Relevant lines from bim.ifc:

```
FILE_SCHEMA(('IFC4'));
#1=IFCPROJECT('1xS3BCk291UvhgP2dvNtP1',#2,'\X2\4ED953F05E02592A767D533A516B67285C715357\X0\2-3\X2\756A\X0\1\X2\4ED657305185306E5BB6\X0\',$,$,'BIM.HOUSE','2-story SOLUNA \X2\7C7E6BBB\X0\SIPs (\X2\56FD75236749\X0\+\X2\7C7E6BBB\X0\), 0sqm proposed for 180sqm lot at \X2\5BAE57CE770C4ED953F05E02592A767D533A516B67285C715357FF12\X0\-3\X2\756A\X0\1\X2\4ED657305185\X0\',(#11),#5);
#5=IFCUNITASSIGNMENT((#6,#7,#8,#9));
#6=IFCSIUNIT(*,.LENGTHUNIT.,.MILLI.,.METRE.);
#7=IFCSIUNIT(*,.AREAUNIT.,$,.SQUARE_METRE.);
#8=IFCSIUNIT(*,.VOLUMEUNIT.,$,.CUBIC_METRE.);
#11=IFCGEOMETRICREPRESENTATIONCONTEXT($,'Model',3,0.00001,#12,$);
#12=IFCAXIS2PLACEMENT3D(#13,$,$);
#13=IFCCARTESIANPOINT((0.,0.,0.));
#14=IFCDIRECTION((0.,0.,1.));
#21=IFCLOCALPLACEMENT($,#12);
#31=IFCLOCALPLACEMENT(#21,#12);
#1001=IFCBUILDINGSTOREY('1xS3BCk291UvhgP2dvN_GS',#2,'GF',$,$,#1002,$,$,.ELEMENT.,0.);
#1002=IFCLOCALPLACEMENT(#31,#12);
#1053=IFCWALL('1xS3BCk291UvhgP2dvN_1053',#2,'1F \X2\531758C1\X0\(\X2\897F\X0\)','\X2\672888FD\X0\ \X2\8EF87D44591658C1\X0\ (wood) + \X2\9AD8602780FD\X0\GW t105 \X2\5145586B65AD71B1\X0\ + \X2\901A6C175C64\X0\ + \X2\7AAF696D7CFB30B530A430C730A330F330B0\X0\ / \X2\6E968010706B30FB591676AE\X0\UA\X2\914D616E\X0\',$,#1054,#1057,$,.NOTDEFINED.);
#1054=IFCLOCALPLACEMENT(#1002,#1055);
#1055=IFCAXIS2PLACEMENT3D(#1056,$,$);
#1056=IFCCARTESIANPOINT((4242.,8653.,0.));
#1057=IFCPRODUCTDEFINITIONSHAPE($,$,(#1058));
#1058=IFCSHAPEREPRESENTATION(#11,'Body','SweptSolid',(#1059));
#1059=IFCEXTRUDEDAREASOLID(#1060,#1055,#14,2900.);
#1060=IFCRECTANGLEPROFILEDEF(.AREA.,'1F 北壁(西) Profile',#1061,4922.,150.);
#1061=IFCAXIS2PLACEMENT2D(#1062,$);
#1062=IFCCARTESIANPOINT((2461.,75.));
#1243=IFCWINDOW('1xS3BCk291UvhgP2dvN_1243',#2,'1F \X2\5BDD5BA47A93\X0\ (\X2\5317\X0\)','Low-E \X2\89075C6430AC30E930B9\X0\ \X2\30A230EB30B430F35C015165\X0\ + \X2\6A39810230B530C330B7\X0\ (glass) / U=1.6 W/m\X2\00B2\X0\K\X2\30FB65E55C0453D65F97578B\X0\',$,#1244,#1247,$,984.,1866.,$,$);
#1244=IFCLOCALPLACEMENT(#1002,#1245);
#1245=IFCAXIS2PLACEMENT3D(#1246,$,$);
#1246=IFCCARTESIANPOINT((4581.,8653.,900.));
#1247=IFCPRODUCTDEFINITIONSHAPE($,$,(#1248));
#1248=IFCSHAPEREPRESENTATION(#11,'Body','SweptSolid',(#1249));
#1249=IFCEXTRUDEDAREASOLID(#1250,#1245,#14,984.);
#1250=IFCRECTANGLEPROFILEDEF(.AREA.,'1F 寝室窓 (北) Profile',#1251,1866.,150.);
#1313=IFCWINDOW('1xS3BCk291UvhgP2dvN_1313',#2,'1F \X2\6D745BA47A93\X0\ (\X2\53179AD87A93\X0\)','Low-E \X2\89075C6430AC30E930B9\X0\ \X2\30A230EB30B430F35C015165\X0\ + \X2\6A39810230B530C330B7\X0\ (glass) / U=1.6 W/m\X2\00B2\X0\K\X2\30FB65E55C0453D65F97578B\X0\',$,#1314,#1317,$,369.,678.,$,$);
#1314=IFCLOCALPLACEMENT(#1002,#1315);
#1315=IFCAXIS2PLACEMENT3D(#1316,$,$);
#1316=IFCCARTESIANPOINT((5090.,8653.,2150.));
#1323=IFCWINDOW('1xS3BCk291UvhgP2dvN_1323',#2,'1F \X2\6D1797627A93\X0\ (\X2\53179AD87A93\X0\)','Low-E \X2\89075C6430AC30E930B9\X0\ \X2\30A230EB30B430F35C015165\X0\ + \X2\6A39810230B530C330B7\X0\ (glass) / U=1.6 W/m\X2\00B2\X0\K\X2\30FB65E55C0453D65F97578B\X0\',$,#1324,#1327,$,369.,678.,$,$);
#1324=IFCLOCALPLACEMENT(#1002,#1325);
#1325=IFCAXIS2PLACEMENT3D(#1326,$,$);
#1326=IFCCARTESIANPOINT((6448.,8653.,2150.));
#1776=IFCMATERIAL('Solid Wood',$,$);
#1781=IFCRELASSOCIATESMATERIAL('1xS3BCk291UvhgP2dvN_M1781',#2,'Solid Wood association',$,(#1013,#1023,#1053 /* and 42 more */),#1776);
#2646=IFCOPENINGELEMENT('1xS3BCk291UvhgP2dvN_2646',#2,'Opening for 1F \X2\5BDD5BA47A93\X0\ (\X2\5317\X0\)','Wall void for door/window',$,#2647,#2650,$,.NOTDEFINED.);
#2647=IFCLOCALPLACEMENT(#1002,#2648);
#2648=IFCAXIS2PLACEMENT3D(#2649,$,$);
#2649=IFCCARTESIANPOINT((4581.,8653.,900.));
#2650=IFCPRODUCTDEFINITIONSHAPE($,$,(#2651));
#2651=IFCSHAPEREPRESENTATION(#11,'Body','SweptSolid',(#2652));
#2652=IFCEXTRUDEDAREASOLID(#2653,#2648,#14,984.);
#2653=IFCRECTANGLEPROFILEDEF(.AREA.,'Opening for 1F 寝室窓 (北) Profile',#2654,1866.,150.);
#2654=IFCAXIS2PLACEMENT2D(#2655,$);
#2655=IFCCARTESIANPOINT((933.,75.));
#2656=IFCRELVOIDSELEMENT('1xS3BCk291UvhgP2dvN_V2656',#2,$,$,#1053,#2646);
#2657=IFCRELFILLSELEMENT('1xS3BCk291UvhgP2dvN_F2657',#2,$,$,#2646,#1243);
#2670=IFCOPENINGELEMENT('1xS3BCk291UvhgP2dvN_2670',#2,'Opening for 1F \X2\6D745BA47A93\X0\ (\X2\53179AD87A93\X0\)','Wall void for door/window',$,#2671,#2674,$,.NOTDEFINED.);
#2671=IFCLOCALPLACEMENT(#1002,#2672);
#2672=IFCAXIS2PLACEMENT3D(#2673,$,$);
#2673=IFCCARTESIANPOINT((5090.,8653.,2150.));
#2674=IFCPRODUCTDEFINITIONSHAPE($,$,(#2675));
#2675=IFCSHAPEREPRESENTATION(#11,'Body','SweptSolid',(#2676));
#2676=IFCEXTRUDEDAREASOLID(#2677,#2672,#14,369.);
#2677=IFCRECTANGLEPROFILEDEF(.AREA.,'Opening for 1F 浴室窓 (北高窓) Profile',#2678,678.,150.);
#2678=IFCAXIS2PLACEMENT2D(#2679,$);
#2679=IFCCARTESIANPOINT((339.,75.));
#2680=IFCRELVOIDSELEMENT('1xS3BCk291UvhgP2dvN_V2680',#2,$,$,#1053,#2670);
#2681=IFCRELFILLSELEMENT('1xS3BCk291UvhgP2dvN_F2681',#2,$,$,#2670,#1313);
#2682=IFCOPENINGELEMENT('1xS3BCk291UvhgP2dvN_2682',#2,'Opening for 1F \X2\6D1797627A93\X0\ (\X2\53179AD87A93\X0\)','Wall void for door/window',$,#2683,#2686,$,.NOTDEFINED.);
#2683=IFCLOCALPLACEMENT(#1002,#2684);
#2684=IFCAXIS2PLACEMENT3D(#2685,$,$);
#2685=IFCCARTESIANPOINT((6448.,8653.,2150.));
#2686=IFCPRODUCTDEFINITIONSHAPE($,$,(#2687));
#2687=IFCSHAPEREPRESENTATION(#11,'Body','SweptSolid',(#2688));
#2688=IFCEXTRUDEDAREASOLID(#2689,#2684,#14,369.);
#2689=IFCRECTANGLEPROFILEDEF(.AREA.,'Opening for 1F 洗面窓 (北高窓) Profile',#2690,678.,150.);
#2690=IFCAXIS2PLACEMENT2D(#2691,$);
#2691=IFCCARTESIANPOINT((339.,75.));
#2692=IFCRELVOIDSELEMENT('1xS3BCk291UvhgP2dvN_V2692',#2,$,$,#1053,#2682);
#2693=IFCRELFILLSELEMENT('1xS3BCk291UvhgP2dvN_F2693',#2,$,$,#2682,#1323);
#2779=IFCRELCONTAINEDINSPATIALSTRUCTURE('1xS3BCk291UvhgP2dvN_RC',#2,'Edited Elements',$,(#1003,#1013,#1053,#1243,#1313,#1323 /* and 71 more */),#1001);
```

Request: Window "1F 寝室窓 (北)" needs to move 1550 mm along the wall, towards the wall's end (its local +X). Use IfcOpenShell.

```python
import ifcopenshell
import ifcopenshell.api.geometry
import ifcopenshell.util.placement
import ifcopenshell.util.unit

model = ifcopenshell.open("bim.ifc")
unit_scale = ifcopenshell.util.unit.calculate_unit_scale(model)

window = model.by_guid("1xS3BCk291UvhgP2dvN_1243")
opening = window.FillsVoids[0].RelatingOpeningElement
wall = opening.VoidsElements[0].RelatingBuildingElement

wall_matrix = ifcopenshell.util.placement.get_local_placement(wall.ObjectPlacement)
shift = wall_matrix[:3, 0] * 1.55 / unit_scale
before = ifcopenshell.util.placement.get_local_placement(window.ObjectPlacement)[:3, 3].copy()

# The window is not placed relative to its opening, so move both.
for product in (opening, window):
    matrix = ifcopenshell.util.placement.get_local_placement(product.ObjectPlacement)
    matrix[:3, 3] += shift
    ifcopenshell.api.geometry.edit_object_placement(model, product=product, matrix=matrix, is_si=False)

after = ifcopenshell.util.placement.get_local_placement(window.ObjectPlacement)[:3, 3]
print("window moved by", (after - before).round(3) + 0.0)

model.write("bim_updated.ifc")
```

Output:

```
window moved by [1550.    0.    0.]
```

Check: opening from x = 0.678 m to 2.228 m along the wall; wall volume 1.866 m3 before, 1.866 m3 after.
